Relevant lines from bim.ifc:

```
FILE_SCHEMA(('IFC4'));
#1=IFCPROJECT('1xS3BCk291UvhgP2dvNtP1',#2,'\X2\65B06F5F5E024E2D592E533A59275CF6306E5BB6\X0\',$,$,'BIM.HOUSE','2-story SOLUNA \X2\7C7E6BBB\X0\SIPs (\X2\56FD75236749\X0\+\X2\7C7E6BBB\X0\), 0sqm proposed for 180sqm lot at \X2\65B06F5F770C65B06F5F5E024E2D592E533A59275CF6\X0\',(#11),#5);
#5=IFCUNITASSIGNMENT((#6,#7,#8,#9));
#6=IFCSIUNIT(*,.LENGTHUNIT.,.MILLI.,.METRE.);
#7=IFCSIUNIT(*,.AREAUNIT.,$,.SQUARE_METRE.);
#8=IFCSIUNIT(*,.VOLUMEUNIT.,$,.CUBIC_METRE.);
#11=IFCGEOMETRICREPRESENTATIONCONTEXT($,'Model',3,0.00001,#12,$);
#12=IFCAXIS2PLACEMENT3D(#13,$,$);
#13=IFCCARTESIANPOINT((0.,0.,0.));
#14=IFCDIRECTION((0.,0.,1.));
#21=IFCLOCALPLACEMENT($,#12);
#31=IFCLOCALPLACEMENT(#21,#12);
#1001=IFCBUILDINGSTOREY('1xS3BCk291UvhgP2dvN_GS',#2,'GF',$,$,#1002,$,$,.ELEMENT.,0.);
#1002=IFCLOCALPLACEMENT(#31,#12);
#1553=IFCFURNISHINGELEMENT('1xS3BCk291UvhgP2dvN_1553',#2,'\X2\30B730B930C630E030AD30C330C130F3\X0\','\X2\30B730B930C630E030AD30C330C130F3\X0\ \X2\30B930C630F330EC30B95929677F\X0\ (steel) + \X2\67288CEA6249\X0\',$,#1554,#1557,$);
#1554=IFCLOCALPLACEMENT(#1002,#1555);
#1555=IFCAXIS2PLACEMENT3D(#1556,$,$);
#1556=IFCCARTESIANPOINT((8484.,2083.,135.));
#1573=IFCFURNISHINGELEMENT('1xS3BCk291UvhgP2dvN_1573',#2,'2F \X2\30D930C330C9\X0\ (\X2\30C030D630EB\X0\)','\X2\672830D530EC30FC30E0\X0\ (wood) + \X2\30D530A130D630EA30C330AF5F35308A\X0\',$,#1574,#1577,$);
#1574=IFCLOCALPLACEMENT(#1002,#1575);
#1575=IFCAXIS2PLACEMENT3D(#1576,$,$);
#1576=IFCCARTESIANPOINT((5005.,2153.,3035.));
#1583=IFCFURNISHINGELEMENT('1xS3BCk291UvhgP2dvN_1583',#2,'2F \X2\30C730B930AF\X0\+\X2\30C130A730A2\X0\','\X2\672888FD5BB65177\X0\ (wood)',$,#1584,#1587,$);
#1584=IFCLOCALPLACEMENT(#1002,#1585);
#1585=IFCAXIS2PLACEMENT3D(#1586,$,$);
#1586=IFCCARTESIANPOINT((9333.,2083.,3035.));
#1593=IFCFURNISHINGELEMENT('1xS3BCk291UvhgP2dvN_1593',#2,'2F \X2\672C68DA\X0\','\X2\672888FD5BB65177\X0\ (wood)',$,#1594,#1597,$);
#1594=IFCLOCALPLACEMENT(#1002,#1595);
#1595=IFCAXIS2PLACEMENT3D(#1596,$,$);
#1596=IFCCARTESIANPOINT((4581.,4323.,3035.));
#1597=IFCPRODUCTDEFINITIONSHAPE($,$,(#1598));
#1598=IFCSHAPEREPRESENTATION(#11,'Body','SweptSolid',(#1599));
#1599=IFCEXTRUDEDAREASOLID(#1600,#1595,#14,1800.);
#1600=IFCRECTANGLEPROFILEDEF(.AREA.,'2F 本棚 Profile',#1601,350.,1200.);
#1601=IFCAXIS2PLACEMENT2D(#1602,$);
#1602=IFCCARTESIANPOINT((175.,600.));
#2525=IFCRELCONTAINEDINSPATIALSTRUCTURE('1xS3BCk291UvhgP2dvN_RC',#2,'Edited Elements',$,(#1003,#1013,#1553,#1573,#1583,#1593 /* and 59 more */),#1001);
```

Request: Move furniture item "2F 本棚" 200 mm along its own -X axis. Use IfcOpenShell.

```python
import ifcopenshell
import ifcopenshell.api.geometry
import ifcopenshell.util.placement

model = ifcopenshell.open("bim.ifc")

item = model.by_guid("1xS3BCk291UvhgP2dvN_1593")
matrix = ifcopenshell.util.placement.get_local_placement(item.ObjectPlacement)
matrix[:3, 3] -= matrix[:3, 0] * 200.0
ifcopenshell.api.geometry.edit_object_placement(model, product=item, matrix=matrix, is_si=False)

print(ifcopenshell.util.placement.get_local_placement(item.ObjectPlacement).round(3) + 0.0)

model.write("bim_v2.ifc")
```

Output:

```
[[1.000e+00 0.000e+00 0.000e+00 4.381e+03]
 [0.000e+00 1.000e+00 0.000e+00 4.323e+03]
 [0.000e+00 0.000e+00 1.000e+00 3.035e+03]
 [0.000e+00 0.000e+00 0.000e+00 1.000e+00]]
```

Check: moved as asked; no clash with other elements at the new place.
